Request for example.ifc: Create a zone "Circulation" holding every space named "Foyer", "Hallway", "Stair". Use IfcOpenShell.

First a look at what the model holds.

```python
import ifcopenshell

model = ifcopenshell.open("example.ifc")
print(model.schema)
seen = {}
for space in model.by_type("IfcSpace"):
    seen[space.LongName] = seen.get(space.LongName, 0) + 1
for name, count in sorted(seen.items(), key=str):
    print(count, "x", name)
print("zones:", [z.Name for z in model.by_type("IfcZone")][:20])
```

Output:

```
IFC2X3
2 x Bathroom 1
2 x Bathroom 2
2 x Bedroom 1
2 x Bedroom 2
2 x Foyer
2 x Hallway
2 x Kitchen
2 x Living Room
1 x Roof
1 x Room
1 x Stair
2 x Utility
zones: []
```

```python
import ifcopenshell
import ifcopenshell.api.group
import ifcopenshell.api.root

model = ifcopenshell.open("example.ifc")

names = {"Foyer", "Hallway", "Stair"}
spaces = [s for s in model.by_type("IfcSpace") if s.LongName in names]

zone = ifcopenshell.api.root.create_entity(model, ifc_class="IfcZone", name="Circulation")
ifcopenshell.api.group.assign_group(model, products=spaces, group=zone)
print(len(spaces), "spaces in", zone.Name)

model.write("example_v2.ifc")
```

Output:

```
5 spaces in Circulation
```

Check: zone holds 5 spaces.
